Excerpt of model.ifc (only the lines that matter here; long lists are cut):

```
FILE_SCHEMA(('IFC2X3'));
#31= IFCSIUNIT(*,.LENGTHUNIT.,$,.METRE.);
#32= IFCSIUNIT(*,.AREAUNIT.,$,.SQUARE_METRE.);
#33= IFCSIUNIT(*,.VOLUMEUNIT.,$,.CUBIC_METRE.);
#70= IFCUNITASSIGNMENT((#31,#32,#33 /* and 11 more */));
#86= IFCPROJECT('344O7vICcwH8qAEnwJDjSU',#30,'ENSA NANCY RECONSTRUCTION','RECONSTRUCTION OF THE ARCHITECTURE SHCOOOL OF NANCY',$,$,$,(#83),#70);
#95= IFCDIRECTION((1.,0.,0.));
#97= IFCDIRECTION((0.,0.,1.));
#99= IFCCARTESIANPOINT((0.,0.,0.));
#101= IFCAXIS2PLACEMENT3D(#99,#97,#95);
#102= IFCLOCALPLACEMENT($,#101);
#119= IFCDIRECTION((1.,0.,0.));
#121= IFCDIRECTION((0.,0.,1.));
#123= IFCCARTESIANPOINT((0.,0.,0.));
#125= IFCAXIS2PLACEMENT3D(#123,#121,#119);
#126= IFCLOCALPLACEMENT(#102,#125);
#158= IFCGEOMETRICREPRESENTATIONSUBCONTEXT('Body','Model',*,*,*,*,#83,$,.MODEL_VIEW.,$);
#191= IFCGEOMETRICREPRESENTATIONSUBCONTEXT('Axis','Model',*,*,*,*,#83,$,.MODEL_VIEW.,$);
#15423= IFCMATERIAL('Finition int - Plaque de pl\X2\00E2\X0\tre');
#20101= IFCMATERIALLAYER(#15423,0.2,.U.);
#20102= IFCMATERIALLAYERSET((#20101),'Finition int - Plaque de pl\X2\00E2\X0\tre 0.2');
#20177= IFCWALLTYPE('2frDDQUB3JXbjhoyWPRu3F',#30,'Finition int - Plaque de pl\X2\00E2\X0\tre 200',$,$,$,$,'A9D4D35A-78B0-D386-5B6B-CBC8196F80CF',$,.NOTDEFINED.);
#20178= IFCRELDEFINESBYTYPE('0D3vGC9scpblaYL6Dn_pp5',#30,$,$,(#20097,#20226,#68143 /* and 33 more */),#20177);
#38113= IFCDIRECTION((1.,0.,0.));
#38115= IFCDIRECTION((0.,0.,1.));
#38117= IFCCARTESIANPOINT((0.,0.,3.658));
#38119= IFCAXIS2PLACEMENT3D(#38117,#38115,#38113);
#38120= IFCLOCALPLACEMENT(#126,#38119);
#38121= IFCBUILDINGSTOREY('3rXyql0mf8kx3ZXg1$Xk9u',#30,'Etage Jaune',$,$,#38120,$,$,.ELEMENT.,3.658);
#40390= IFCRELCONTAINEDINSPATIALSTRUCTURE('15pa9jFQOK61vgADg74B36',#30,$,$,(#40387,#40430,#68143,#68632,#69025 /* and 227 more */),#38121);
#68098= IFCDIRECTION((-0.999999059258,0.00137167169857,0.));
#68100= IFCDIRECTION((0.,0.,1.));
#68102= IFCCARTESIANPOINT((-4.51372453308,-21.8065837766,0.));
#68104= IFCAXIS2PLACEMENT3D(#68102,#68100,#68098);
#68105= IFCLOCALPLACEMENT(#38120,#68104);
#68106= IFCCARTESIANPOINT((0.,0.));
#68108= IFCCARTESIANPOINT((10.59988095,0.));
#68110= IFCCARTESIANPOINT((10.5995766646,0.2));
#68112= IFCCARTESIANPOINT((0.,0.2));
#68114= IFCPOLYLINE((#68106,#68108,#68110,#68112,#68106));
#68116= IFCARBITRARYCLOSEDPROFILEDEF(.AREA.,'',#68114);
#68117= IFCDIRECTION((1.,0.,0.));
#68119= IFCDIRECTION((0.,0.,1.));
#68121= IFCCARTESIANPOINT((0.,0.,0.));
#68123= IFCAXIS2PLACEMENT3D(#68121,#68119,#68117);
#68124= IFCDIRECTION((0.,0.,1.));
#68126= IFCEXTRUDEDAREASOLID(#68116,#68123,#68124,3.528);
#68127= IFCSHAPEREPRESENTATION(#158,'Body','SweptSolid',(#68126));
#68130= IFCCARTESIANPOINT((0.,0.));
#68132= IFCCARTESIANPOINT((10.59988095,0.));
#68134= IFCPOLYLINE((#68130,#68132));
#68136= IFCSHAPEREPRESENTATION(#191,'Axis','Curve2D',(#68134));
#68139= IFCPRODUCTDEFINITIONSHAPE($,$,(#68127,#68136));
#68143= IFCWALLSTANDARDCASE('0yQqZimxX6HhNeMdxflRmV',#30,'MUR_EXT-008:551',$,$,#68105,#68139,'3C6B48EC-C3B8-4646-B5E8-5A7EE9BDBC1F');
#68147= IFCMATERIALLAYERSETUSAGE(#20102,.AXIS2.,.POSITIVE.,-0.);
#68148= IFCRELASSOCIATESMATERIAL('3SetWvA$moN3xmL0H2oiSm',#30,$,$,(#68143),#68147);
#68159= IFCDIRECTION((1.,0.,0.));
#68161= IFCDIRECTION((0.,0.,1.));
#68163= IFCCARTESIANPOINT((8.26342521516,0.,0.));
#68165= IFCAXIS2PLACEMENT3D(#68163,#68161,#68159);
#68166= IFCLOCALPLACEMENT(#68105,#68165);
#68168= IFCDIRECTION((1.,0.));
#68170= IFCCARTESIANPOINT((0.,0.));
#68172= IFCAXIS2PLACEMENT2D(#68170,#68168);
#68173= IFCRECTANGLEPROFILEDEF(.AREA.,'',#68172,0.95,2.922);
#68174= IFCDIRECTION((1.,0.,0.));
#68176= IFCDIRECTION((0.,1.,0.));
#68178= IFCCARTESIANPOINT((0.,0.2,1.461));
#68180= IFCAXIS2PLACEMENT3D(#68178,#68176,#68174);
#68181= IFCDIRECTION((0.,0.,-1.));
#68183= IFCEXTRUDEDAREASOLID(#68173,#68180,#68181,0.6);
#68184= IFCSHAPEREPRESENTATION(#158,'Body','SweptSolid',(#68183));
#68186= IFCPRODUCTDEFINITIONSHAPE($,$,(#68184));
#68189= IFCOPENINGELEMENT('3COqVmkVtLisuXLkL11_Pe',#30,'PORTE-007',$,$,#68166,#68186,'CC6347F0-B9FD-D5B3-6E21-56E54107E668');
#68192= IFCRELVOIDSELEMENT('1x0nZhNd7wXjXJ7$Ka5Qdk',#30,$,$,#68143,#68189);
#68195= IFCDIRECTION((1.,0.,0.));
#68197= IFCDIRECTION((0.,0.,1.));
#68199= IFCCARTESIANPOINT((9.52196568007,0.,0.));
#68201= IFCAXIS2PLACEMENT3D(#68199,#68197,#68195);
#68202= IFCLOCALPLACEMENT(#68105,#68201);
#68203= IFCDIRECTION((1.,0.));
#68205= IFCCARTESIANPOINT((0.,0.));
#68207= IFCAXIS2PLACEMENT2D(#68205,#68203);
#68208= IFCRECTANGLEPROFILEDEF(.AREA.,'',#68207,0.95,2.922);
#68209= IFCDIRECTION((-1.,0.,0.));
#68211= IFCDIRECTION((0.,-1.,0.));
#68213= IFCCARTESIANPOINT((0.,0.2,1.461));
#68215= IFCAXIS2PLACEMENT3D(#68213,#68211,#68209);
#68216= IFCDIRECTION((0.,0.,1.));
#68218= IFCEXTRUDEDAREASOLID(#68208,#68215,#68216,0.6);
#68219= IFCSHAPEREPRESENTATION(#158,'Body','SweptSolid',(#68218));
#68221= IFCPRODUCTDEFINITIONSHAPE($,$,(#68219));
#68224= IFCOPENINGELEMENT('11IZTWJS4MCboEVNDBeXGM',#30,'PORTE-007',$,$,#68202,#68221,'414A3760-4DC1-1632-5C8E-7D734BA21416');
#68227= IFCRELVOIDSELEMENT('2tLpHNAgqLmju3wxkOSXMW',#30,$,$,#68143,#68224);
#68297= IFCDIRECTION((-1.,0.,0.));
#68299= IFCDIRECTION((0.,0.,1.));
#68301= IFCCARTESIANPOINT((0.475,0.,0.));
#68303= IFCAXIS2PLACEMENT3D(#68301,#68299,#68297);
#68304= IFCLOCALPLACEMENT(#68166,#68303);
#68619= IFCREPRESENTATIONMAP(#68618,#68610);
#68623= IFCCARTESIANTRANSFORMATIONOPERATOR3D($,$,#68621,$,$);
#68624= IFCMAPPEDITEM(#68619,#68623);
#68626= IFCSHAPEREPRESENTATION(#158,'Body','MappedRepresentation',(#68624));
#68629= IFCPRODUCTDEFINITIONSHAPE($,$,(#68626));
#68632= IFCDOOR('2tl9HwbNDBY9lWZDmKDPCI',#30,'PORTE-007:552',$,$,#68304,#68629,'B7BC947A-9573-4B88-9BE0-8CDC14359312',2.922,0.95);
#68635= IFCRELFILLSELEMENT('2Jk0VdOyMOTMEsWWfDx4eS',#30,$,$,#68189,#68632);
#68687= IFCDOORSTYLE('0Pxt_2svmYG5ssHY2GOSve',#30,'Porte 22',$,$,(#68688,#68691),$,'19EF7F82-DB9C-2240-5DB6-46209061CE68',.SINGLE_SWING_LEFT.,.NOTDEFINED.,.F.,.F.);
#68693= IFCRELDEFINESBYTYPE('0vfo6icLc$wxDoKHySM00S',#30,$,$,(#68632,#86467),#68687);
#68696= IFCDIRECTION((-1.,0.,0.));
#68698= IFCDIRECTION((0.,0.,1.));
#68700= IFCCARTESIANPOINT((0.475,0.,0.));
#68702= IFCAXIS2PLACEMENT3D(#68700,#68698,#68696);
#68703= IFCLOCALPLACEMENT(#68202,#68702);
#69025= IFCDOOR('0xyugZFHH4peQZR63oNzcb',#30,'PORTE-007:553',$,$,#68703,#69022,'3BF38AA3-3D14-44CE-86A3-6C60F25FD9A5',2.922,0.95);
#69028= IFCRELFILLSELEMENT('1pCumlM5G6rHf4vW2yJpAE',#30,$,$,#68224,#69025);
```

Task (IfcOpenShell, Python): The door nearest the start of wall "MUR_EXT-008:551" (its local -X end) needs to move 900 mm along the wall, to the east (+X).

```python
import ifcopenshell
import ifcopenshell.api.geometry
import ifcopenshell.util.placement
import ifcopenshell.util.unit

model = ifcopenshell.open("model.ifc")
unit_scale = ifcopenshell.util.unit.calculate_unit_scale(model)

door = model.by_id(68632)
opening = door.FillsVoids[0].RelatingOpeningElement
wall = opening.VoidsElements[0].RelatingBuildingElement

wall_matrix = ifcopenshell.util.placement.get_local_placement(wall.ObjectPlacement)
shift = wall_matrix[:3, 0] * -0.9 / unit_scale
before = ifcopenshell.util.placement.get_local_placement(door.ObjectPlacement)[:3, 3].copy()

# The door is placed relative to its opening, so it follows when the opening moves.
matrix = ifcopenshell.util.placement.get_local_placement(opening.ObjectPlacement)
matrix[:3, 3] += shift
ifcopenshell.api.geometry.edit_object_placement(
    model, product=opening, matrix=matrix, is_si=False, should_transform_children=True
)

after = ifcopenshell.util.placement.get_local_placement(door.ObjectPlacement)[:3, 3]
print("door moved by", (after - before).round(3) + 0.0)

model.write("model_v2.ifc")
```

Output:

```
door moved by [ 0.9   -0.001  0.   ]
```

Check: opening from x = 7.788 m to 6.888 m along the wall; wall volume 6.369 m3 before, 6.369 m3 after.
